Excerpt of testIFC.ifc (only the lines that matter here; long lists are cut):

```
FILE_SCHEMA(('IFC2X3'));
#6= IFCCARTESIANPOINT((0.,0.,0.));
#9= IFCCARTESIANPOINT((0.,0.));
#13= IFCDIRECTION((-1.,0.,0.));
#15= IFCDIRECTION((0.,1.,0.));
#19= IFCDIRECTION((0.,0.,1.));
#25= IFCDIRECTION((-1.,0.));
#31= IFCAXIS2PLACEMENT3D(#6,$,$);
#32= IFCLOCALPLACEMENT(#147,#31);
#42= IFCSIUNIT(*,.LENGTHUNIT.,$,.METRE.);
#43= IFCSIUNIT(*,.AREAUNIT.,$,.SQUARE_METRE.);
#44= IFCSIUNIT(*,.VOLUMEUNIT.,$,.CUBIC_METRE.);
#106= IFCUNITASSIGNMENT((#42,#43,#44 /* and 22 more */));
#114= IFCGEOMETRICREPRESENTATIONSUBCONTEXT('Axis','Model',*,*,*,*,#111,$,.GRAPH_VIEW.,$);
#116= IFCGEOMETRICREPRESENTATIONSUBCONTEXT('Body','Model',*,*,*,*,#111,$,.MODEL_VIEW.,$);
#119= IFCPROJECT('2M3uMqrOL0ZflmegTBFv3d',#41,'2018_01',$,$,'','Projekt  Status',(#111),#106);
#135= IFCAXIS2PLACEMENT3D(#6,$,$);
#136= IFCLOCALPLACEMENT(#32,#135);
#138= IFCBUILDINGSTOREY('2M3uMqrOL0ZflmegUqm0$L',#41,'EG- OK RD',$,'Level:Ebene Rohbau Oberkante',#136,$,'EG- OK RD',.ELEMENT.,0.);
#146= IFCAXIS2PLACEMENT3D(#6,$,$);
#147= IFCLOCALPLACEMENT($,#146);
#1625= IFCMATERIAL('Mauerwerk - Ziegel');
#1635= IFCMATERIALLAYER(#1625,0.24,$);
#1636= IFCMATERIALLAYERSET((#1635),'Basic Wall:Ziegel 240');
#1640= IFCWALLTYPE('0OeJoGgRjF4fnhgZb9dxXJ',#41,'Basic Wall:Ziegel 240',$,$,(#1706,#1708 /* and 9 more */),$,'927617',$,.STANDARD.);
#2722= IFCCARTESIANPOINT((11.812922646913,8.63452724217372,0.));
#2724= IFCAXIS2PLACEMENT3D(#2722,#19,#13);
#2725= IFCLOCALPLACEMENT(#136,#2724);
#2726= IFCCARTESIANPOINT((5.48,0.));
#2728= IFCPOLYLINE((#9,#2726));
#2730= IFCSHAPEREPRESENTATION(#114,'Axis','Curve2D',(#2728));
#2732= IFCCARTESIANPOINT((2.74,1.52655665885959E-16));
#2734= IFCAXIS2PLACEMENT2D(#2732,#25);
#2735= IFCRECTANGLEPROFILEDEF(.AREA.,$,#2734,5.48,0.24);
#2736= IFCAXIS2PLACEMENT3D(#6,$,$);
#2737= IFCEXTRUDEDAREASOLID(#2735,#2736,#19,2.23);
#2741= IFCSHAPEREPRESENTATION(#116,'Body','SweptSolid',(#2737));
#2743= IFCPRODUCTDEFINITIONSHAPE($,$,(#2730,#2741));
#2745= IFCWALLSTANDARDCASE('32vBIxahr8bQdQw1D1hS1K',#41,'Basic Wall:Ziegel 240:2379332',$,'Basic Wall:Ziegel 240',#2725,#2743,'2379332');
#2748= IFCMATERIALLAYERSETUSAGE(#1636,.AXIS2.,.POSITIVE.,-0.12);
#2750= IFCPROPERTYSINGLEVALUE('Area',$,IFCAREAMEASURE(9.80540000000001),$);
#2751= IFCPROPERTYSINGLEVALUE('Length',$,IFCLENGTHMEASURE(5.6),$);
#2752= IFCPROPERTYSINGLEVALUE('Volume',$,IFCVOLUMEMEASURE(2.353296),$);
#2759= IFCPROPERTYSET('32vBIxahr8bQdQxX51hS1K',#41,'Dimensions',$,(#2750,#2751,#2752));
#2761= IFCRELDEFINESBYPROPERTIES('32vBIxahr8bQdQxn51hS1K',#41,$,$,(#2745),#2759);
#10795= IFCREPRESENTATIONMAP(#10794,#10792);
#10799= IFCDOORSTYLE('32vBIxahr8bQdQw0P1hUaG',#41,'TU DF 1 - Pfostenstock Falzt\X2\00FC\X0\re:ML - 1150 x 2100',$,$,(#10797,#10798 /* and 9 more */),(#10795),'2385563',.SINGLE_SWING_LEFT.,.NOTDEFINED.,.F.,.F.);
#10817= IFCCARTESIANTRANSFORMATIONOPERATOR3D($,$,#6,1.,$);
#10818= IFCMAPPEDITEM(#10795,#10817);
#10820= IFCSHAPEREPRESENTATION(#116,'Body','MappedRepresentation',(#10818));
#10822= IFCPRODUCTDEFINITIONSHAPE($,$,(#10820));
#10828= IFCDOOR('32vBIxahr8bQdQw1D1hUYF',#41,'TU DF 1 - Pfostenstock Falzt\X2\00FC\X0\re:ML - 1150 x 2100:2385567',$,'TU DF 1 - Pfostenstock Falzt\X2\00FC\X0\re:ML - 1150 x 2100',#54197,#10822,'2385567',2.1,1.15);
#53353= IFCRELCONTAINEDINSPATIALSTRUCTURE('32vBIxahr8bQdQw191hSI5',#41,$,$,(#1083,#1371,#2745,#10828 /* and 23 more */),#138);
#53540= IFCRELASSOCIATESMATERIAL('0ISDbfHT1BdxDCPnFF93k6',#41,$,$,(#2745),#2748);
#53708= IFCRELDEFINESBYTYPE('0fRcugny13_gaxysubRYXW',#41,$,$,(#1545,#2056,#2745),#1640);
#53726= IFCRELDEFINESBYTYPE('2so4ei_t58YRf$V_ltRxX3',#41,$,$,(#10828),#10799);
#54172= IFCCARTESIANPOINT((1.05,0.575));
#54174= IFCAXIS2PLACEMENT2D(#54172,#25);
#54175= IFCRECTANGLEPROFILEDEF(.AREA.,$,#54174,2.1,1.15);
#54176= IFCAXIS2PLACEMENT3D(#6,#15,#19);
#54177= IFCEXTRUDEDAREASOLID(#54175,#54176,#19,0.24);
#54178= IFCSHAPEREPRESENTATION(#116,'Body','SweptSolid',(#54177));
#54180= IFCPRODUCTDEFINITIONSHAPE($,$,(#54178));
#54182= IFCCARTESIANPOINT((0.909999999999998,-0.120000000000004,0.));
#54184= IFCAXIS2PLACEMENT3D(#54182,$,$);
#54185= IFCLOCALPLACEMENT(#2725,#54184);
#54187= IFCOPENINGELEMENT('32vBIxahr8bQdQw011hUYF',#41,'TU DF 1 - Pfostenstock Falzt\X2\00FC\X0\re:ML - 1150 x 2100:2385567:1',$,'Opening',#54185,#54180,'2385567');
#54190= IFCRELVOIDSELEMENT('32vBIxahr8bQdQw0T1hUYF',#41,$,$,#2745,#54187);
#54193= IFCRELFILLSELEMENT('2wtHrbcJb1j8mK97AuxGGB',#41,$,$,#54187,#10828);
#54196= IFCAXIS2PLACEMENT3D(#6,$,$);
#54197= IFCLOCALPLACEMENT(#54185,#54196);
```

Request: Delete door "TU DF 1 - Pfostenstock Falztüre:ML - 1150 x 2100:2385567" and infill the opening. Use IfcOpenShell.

```python
import ifcopenshell
import ifcopenshell.api.feature
import ifcopenshell.api.pset
import ifcopenshell.api.root
import ifcopenshell.geom
import ifcopenshell.util.element
import ifcopenshell.util.shape
import ifcopenshell.util.unit

model = ifcopenshell.open("testIFC.ifc")
area_scale = ifcopenshell.util.unit.calculate_unit_scale(model, "AREAUNIT")
volume_scale = ifcopenshell.util.unit.calculate_unit_scale(model, "VOLUMEUNIT")
settings = ifcopenshell.geom.settings()


def volume(element):
    """Net volume in cubic metres, openings subtracted."""
    shape = ifcopenshell.geom.create_shape(settings, element)
    return ifcopenshell.util.shape.get_volume(shape.geometry)


door = model.by_guid("32vBIxahr8bQdQw1D1hUYF")
opening = door.FillsVoids[0].RelatingOpeningElement
wall = opening.VoidsElements[0].RelatingBuildingElement
before = volume(wall)

ifcopenshell.api.root.remove_product(model, product=door)
ifcopenshell.api.feature.remove_feature(model, feature=opening)

after = volume(wall)
thickness = 0.24  # wall thickness in metres

# Update the wall's stored quantities.
pset = model.by_id(ifcopenshell.util.element.get_pset(wall, "Dimensions", should_inherit=False)["id"])
ifcopenshell.api.pset.edit_pset(model, pset=pset, properties={
    "Area": model.create_entity("IfcAreaMeasure", after / thickness / area_scale),
    "Volume": model.create_entity("IfcVolumeMeasure", after / volume_scale),
})

print(f"wall volume {before:.3f} -> {after:.3f} m3")

model.write("testIFC_updated.ifc")
```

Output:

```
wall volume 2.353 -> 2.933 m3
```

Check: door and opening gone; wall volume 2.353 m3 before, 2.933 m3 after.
